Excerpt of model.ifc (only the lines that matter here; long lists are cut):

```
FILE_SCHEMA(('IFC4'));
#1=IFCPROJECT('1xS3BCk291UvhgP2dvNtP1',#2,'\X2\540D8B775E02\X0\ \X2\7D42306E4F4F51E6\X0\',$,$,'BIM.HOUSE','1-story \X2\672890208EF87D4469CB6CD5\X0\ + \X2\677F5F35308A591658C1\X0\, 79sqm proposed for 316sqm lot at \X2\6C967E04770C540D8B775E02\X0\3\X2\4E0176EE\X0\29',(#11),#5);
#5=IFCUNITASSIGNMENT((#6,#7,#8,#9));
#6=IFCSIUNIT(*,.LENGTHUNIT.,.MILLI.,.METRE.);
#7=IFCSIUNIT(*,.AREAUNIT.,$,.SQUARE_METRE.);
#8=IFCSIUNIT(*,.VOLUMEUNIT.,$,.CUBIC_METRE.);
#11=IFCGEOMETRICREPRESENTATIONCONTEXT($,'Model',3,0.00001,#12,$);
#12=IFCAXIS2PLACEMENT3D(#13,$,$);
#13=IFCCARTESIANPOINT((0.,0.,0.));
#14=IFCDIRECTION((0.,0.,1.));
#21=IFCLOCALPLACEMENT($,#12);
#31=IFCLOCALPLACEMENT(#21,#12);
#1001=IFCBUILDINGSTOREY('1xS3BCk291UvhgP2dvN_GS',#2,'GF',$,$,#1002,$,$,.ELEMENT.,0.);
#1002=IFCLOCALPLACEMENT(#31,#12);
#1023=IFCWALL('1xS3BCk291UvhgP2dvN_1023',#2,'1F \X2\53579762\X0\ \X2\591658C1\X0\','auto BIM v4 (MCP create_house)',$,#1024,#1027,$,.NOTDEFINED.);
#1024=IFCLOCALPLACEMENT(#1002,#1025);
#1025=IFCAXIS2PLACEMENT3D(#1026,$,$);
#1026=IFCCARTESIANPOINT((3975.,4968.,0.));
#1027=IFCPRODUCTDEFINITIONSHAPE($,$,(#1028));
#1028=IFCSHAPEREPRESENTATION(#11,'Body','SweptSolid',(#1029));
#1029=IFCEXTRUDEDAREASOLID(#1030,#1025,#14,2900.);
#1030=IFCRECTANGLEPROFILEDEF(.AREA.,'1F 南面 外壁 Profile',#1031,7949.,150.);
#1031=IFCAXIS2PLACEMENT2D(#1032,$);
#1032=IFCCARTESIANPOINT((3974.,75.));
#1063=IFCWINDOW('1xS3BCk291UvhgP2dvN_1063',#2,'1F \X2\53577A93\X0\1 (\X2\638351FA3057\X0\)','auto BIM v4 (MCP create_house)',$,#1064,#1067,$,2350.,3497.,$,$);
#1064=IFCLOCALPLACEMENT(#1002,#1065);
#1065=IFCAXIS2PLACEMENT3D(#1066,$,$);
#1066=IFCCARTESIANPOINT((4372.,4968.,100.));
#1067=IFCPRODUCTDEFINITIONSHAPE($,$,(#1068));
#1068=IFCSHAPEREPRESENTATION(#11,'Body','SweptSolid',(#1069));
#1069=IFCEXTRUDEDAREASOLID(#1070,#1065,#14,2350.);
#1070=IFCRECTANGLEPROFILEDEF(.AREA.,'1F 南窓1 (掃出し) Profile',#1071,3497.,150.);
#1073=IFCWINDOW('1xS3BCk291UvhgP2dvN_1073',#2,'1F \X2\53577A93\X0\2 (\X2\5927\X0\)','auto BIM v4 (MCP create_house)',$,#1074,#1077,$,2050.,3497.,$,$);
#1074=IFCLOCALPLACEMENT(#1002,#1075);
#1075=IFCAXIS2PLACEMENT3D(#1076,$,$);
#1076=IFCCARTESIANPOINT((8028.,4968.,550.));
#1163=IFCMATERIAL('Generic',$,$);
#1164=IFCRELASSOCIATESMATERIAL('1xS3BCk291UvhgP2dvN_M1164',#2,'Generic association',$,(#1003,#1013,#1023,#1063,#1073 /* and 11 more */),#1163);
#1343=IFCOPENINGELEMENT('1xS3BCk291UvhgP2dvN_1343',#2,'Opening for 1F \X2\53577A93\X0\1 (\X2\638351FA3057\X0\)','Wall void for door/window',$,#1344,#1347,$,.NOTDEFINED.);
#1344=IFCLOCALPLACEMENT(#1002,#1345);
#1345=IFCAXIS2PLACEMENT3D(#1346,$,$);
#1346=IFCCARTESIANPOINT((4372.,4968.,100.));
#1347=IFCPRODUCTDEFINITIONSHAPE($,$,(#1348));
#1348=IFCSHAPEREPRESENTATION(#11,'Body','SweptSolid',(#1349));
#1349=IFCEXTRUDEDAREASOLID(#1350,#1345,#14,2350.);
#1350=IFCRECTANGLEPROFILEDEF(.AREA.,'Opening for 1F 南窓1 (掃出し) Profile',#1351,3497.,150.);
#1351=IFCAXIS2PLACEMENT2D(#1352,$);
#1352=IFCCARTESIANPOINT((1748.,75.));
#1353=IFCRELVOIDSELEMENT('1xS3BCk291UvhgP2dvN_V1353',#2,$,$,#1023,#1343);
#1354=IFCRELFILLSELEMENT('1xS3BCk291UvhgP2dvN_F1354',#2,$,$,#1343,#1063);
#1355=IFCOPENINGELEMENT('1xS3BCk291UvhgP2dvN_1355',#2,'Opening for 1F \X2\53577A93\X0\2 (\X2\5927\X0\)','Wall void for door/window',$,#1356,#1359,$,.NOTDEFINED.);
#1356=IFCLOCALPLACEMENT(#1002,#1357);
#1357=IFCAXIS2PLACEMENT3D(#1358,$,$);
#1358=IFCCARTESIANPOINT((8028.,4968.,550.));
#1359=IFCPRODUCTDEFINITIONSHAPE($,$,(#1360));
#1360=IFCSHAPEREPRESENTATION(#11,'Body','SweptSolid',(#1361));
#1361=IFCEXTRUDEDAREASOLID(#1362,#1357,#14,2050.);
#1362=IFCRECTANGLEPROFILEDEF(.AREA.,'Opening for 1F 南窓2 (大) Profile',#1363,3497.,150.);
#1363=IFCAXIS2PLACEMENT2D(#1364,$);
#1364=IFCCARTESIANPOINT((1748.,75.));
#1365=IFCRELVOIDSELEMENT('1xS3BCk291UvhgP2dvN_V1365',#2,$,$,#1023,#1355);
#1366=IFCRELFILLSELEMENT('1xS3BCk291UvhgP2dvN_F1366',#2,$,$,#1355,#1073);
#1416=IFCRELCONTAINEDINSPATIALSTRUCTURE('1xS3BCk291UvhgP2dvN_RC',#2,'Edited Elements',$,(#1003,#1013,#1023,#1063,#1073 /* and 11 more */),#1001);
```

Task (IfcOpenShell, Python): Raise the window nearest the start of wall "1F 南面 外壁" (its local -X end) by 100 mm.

```python
import numpy as np
import ifcopenshell
import ifcopenshell.api.geometry
import ifcopenshell.util.placement
import ifcopenshell.util.unit

model = ifcopenshell.open("model.ifc")
unit_scale = ifcopenshell.util.unit.calculate_unit_scale(model)

window = model.by_id(1063)
opening = window.FillsVoids[0].RelatingOpeningElement
dz = 0.1 / unit_scale

shift = np.array([0.0, 0.0, dz])
# The window is not placed relative to its opening, so move both.
for product in (opening, window):
    matrix = ifcopenshell.util.placement.get_local_placement(product.ObjectPlacement)
    matrix[:3, 3] += shift
    ifcopenshell.api.geometry.edit_object_placement(model, product=product, matrix=matrix, is_si=False)

print(f"moved by {dz * unit_scale:+.3f} m")

model.write("model_v2.ifc")
```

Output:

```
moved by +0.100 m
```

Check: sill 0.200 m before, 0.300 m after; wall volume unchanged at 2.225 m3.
